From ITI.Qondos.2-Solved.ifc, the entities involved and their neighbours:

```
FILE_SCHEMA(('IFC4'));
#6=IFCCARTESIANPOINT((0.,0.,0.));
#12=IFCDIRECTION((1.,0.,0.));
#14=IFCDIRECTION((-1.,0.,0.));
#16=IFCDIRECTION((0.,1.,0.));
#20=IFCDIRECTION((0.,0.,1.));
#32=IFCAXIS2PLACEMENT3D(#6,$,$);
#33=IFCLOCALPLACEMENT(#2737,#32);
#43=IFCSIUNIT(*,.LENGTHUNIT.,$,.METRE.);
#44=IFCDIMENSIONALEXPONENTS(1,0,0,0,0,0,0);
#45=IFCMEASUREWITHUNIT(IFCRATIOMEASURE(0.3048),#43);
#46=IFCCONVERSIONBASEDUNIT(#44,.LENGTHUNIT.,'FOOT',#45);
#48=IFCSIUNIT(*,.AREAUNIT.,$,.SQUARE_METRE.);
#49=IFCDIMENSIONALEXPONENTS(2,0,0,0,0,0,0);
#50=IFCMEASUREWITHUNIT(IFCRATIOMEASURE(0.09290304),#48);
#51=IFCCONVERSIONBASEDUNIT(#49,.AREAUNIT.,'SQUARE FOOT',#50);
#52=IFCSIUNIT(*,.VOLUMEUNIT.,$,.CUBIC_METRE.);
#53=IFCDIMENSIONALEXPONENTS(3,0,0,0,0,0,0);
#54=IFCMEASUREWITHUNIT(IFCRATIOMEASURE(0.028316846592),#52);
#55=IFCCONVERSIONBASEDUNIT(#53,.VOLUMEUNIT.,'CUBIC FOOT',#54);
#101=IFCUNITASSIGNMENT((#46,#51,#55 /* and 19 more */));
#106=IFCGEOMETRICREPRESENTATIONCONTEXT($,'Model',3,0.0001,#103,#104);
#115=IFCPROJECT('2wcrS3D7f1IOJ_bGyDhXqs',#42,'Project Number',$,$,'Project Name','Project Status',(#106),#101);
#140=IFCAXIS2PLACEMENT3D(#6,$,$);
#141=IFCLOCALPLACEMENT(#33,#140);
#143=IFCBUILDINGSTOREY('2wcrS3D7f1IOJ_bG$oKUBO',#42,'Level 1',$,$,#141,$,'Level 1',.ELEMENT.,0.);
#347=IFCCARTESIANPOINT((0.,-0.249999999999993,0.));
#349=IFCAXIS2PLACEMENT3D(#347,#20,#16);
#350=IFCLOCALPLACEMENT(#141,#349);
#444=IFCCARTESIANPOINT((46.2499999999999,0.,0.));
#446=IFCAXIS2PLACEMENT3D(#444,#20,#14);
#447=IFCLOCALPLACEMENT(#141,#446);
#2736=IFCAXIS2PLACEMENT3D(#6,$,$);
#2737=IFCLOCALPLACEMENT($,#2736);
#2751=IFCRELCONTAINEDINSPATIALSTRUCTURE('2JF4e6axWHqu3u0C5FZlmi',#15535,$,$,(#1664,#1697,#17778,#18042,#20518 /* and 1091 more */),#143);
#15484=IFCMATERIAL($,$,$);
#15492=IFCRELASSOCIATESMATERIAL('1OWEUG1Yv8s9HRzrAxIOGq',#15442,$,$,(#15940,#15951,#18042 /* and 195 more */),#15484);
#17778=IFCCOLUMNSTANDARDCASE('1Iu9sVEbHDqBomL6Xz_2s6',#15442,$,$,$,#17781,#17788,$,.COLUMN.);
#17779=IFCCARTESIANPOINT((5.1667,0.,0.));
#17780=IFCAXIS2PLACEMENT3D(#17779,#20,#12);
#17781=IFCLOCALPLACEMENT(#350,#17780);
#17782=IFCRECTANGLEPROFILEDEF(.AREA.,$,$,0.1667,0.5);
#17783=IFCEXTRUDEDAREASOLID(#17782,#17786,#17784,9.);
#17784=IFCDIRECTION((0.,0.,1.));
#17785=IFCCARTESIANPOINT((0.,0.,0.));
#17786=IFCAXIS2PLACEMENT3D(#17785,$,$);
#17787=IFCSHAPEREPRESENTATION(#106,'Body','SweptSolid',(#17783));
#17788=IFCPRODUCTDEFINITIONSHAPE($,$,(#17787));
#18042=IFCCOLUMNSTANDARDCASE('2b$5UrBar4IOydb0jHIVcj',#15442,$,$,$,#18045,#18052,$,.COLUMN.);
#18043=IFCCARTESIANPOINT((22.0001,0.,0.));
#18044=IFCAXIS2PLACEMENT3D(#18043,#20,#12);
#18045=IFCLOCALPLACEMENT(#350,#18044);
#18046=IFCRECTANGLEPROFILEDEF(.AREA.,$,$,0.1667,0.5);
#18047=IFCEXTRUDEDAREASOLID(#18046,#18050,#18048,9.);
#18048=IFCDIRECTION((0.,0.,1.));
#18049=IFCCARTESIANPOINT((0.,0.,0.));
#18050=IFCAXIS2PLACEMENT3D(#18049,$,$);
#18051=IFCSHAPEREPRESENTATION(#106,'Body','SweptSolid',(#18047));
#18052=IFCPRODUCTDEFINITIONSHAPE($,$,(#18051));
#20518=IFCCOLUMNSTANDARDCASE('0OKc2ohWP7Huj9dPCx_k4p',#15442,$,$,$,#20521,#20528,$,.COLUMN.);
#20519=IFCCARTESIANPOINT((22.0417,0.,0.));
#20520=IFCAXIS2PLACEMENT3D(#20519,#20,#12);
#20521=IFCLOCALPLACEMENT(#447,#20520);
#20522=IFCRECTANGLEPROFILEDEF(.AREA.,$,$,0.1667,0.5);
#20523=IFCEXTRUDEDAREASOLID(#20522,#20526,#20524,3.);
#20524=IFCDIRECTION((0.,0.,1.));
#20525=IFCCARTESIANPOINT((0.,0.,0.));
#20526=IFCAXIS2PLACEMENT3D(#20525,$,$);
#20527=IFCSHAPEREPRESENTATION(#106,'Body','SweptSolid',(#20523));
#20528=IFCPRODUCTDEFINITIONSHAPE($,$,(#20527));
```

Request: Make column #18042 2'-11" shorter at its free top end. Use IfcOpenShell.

```python
import ifcopenshell
import ifcopenshell.util.unit

model = ifcopenshell.open("ITI.Qondos.2-Solved.ifc")
unit_scale = ifcopenshell.util.unit.calculate_unit_scale(model)

member = model.by_guid("2b$5UrBar4IOydb0jHIVcj")
change = -35 * 0.0254 / unit_scale

# The extrusion runs towards the end named, so only its depth changes.
body = next(r for r in member.Representation.Representations if r.RepresentationIdentifier == "Body")
solid = body.Items[0]
old_length = solid.Depth
solid.Depth += change

print(f"length {old_length:g} -> {solid.Depth:g}")

model.write("ITI.Qondos.2-Solved_v2.ifc")
```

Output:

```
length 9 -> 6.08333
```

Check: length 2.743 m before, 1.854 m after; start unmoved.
